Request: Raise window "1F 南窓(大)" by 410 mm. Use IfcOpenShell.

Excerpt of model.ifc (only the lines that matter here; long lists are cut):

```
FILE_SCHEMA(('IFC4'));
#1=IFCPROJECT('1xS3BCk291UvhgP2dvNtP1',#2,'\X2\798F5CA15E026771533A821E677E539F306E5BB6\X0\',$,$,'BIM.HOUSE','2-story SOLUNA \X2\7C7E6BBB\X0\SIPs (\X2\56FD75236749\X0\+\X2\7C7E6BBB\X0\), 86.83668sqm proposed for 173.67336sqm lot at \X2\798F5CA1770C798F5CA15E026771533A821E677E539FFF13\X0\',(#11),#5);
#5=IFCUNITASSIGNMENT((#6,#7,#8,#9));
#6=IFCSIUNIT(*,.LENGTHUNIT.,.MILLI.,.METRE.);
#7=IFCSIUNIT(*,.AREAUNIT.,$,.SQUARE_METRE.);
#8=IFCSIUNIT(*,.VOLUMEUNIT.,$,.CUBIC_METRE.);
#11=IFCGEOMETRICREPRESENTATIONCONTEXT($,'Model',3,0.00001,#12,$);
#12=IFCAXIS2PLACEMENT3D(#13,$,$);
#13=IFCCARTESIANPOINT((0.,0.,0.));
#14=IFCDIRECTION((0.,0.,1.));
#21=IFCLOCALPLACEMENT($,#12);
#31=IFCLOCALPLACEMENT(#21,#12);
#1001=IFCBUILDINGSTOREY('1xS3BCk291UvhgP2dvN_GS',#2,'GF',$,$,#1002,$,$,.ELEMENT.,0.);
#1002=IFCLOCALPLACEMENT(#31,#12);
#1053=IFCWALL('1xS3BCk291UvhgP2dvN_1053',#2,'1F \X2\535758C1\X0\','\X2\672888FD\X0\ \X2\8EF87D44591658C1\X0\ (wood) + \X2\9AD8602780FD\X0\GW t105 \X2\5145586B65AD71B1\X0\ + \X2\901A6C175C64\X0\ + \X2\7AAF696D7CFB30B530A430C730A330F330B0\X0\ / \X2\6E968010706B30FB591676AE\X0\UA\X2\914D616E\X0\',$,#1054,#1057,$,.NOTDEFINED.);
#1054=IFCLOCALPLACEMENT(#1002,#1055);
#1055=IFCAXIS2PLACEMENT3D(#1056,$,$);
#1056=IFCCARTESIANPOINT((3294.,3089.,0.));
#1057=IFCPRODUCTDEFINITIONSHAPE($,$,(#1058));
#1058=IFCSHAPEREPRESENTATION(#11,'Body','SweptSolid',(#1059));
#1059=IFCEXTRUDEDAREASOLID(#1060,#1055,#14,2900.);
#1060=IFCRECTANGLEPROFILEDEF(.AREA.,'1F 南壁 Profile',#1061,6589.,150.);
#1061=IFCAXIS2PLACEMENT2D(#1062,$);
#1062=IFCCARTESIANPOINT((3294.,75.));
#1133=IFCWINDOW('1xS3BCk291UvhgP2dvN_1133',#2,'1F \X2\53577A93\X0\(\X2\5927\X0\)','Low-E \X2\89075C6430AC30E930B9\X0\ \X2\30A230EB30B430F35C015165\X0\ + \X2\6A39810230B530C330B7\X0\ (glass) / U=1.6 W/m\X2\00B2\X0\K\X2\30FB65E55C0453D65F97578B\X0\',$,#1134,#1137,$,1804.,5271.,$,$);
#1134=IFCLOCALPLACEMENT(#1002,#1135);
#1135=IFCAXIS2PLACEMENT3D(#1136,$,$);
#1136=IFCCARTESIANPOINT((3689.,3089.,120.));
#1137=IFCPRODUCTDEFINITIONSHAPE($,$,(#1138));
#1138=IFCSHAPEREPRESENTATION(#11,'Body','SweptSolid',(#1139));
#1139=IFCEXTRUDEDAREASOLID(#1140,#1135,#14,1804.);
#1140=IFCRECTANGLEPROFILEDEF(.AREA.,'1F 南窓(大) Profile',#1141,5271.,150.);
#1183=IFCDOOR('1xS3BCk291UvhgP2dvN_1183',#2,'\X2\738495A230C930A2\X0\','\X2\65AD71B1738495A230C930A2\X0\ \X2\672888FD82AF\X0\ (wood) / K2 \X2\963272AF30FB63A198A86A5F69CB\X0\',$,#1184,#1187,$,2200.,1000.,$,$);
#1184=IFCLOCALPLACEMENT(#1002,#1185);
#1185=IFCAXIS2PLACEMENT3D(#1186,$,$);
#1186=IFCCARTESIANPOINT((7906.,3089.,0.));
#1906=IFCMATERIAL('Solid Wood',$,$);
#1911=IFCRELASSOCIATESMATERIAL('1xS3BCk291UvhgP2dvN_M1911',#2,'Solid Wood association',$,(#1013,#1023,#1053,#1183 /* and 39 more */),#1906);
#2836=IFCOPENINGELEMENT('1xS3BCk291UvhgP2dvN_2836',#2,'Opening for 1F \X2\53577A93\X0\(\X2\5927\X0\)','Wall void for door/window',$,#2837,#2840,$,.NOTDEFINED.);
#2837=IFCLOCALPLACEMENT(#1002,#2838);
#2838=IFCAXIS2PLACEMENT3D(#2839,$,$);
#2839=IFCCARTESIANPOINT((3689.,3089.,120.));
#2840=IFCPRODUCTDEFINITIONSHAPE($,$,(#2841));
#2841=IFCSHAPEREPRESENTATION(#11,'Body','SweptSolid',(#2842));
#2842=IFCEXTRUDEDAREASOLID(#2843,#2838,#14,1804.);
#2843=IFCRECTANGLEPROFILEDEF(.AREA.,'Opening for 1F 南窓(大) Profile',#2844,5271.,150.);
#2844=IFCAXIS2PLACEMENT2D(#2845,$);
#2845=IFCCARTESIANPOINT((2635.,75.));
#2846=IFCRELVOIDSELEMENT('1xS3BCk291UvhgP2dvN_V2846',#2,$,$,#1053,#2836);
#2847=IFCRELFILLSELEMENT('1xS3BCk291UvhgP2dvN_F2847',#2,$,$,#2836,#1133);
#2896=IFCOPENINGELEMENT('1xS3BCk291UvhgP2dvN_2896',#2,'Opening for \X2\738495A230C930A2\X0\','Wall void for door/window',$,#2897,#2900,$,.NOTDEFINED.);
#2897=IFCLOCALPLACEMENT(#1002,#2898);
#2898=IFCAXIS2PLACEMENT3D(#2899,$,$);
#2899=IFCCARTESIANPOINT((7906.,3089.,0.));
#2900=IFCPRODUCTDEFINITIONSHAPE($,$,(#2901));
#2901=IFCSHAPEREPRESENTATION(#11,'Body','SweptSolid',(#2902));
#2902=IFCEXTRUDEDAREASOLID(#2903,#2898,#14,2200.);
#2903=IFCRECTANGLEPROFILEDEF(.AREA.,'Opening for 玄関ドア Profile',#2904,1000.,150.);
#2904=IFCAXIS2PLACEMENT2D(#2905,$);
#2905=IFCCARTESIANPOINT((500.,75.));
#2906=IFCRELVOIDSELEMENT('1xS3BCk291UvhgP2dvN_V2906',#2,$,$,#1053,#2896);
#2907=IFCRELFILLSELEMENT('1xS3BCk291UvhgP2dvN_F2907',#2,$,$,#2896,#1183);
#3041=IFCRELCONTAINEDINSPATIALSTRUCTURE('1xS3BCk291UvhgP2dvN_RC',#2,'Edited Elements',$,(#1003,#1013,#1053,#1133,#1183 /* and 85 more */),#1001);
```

```python
import numpy as np
import ifcopenshell
import ifcopenshell.api.geometry
import ifcopenshell.util.placement
import ifcopenshell.util.unit

model = ifcopenshell.open("model.ifc")
unit_scale = ifcopenshell.util.unit.calculate_unit_scale(model)

window = model.by_guid("1xS3BCk291UvhgP2dvN_1133")
opening = window.FillsVoids[0].RelatingOpeningElement
dz = 410.0

shift = np.array([0.0, 0.0, dz])
# The window is not placed relative to its opening, so move both.
for product in (opening, window):
    matrix = ifcopenshell.util.placement.get_local_placement(product.ObjectPlacement)
    matrix[:3, 3] += shift
    ifcopenshell.api.geometry.edit_object_placement(model, product=product, matrix=matrix, is_si=False)

print(f"moved by {dz * unit_scale:+.3f} m")

model.write("model_edited.ifc")
```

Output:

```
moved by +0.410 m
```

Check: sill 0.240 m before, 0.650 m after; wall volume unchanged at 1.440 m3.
